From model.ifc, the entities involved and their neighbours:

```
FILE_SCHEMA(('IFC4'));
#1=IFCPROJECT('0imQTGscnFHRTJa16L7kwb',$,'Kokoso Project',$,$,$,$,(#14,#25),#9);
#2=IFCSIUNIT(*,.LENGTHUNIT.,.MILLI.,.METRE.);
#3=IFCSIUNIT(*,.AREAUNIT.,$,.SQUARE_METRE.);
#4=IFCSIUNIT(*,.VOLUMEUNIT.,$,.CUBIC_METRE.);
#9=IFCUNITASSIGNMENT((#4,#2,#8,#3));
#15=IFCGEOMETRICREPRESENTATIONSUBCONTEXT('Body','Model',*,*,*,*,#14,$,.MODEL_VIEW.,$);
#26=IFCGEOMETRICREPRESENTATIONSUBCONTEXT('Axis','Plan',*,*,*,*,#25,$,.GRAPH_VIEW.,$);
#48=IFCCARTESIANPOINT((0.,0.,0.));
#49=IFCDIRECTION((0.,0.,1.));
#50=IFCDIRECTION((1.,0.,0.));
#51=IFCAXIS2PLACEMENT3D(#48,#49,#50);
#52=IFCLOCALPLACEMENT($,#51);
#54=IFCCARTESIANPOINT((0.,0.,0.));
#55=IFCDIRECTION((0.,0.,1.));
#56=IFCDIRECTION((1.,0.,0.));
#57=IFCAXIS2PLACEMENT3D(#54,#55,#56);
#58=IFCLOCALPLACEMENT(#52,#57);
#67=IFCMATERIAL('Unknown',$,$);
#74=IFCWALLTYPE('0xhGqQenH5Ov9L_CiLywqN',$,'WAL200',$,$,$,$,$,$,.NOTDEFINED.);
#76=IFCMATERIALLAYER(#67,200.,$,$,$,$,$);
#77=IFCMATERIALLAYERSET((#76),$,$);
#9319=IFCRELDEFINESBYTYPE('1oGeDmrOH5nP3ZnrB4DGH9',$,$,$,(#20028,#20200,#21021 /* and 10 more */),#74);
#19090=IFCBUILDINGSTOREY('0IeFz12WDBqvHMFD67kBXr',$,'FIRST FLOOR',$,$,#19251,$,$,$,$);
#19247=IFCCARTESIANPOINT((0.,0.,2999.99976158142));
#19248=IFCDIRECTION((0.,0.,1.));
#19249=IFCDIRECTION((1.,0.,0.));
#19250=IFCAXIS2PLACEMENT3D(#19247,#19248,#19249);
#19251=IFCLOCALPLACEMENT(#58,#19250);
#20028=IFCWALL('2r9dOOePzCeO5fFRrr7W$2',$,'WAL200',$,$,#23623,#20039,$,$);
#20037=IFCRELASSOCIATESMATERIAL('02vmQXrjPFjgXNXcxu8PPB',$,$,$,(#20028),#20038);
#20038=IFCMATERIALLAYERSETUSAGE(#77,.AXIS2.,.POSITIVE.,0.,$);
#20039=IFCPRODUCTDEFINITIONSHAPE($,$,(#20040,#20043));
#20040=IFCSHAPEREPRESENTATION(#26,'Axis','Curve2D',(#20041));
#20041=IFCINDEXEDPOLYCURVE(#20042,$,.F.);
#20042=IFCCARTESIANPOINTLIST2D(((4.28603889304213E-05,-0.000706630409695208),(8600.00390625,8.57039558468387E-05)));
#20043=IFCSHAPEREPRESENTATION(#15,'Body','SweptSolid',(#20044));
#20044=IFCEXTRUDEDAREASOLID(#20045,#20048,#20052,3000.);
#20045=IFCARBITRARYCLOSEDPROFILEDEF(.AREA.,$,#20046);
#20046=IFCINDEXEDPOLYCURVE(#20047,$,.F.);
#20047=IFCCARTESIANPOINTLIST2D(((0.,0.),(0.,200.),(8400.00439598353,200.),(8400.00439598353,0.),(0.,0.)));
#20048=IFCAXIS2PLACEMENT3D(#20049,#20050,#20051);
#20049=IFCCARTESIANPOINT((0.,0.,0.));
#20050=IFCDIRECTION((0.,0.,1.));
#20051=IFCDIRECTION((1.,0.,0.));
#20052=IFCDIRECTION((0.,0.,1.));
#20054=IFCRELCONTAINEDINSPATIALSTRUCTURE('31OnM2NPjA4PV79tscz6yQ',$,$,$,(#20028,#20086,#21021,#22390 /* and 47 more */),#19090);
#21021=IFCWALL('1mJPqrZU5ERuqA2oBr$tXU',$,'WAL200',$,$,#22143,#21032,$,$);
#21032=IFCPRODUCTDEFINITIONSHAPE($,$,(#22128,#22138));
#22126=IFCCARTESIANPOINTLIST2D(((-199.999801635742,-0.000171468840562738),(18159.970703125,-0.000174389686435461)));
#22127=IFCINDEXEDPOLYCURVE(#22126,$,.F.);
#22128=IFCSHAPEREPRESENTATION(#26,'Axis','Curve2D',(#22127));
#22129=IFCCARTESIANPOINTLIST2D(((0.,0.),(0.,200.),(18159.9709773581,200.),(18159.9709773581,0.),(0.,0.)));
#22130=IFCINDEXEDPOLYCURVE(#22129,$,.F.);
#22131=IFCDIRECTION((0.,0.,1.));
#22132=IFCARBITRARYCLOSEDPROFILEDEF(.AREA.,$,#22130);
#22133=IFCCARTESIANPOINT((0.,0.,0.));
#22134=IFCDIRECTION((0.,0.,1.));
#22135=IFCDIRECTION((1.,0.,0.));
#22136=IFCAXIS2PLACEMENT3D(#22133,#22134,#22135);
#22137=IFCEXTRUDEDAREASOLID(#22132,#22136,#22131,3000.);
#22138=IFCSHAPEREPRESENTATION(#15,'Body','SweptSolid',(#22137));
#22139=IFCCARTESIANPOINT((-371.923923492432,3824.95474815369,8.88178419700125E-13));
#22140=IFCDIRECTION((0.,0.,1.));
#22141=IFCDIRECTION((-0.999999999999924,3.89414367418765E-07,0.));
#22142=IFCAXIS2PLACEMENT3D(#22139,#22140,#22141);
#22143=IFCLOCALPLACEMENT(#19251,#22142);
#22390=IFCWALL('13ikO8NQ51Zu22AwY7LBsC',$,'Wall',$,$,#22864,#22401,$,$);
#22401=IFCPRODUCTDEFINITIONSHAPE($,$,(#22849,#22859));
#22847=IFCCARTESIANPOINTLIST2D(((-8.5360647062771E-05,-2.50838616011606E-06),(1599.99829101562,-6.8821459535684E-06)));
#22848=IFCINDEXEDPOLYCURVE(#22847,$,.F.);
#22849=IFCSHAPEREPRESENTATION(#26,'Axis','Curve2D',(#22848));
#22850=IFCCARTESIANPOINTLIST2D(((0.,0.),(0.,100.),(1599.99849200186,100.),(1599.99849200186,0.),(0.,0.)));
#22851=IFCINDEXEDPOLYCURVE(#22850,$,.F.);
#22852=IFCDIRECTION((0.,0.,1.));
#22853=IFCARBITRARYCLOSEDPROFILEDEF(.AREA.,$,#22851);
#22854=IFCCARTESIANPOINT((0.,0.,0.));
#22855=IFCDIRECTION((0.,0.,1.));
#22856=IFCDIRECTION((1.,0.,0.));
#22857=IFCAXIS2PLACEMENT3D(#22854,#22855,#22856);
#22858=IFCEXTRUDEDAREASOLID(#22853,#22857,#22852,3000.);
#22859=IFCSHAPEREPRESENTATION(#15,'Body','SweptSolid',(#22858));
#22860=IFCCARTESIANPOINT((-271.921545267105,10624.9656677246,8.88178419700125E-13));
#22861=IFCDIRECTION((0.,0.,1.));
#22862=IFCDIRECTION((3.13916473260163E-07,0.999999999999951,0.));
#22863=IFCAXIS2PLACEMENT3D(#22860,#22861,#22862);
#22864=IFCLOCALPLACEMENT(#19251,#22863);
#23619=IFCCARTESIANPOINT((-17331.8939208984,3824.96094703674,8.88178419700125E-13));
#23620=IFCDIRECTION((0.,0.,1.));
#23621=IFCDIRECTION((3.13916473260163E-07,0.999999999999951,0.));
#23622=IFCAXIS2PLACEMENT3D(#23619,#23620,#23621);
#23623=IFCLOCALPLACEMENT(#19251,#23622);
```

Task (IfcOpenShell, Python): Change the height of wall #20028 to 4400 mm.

```python
import ifcopenshell
import ifcopenshell.geom
import ifcopenshell.util.representation
import ifcopenshell.util.shape
import ifcopenshell.util.unit

model = ifcopenshell.open("model.ifc")
unit_scale = ifcopenshell.util.unit.calculate_unit_scale(model)
settings = ifcopenshell.geom.settings()


def volume(element):
    """Net volume in cubic metres, openings subtracted."""
    shape = ifcopenshell.geom.create_shape(settings, element)
    return ifcopenshell.util.shape.get_volume(shape.geometry)


wall = model.by_guid("2r9dOOePzCeO5fFRrr7W$2")
before = volume(wall)

body = ifcopenshell.util.representation.get_representation(wall, "Model", "Body")
solid = body.Items[0]
old_height = solid.Depth
solid.Depth = 4.4 / unit_scale
after = volume(wall)

print(f"height {old_height:g} -> {solid.Depth:g}, volume {before:.3f} -> {after:.3f} m3")

model.write("model-out.ifc")
```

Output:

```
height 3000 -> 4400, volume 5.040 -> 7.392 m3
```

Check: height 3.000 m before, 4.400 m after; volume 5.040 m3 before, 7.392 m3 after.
